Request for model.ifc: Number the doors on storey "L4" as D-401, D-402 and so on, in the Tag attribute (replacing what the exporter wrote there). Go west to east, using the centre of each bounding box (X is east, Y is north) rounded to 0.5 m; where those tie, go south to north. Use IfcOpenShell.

First a look at what the model holds.

```python
import ifcopenshell
import ifcopenshell.util.element
import ifcopenshell.util.placement

model = ifcopenshell.open("model.ifc")
print(model.schema)
storey = next(s for s in model.by_type("IfcBuildingStorey") if s.Name == "L4")
doors = [e for e in ifcopenshell.util.element.get_decomposition(storey) if e.is_a("IfcDoor")]
for e in sorted(doors, key=lambda e: e.id()):
    origin = ifcopenshell.util.placement.get_local_placement(e.ObjectPlacement)[:3, 3]
    print(e.id(), e.Tag, e.Name, origin.round(2) + 0.0, sep=" | ")
```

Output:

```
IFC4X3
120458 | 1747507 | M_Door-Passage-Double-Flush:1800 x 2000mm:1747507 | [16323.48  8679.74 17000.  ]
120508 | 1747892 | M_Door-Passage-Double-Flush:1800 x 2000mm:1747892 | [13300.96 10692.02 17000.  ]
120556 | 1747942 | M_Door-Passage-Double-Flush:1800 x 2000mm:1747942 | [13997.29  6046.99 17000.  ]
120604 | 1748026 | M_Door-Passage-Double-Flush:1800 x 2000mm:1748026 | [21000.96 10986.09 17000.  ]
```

```python
import ifcopenshell
import ifcopenshell.geom
import ifcopenshell.util.element
import ifcopenshell.util.shape

model = ifcopenshell.open("model.ifc")
settings = ifcopenshell.geom.settings()
settings.set("use-world-coords", True)


def centre(element):
    shape = ifcopenshell.geom.create_shape(settings, element)
    return ifcopenshell.util.shape.get_bbox_centroid(shape.geometry)


storey = next(s for s in model.by_type("IfcBuildingStorey") if s.Name == "L4")
doors = [e for e in ifcopenshell.util.element.get_decomposition(storey) if e.is_a("IfcDoor")]

# Insertion points can sit at a corner or the storey origin, so sort by the geometry (in metres).
centres = {e: centre(e) for e in doors}
doors.sort(key=lambda e: (round(centres[e][0] / 0.5), centres[e][1]))

for i, e in enumerate(doors, start=1):
    number = f"D-4{i:02d}"
    e.Tag = number
    print(e.id(), number)

model.write("model_updated.ifc")
```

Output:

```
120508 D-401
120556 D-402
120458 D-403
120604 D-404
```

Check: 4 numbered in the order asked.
